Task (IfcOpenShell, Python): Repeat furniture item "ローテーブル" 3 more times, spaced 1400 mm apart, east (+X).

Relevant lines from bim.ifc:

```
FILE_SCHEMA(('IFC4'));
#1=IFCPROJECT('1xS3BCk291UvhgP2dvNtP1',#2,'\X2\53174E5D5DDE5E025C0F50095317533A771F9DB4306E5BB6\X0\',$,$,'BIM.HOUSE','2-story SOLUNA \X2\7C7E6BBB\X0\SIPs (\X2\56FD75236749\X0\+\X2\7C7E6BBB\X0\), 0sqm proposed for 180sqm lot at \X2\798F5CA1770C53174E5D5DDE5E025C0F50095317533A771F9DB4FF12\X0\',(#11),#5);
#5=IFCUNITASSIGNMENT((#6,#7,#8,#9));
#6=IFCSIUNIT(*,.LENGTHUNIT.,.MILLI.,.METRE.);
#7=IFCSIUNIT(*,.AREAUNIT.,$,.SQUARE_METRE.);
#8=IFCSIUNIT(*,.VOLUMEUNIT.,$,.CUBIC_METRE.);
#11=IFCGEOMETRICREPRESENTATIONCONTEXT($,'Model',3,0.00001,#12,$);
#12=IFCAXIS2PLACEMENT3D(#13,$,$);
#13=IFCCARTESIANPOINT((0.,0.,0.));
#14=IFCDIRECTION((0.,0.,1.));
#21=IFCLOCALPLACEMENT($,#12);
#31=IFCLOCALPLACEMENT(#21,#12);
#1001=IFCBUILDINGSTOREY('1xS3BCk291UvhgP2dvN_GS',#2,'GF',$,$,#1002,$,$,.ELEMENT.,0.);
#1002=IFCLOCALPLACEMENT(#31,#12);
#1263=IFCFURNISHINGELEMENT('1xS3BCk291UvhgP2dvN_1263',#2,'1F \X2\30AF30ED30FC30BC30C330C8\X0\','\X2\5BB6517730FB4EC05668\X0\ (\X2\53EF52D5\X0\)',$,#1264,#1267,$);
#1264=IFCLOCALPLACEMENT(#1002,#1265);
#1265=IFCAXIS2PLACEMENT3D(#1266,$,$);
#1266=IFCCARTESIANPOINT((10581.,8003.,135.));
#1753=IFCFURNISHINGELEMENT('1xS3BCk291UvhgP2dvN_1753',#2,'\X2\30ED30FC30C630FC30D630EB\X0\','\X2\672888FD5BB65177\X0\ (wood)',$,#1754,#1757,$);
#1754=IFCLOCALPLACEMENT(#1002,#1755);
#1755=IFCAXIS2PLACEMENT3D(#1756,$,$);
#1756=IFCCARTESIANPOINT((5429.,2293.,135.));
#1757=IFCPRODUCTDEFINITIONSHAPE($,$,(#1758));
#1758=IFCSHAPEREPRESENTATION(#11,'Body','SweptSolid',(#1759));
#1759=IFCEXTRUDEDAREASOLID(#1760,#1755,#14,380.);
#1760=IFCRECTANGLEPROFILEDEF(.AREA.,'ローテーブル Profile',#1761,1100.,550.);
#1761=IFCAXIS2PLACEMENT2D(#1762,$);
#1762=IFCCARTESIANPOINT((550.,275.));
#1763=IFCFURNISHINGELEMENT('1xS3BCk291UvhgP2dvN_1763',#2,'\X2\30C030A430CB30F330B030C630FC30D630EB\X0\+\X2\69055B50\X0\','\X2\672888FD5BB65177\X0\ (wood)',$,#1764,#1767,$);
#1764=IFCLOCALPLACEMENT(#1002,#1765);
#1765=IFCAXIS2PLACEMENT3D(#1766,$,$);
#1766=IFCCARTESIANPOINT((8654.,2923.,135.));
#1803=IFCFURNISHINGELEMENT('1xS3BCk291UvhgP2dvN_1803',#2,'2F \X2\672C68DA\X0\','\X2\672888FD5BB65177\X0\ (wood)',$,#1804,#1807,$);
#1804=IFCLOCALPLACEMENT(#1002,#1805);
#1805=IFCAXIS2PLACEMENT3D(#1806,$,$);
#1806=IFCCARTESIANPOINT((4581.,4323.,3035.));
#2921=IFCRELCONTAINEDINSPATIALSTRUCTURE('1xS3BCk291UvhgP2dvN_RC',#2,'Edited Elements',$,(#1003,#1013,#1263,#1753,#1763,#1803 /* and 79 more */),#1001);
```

```python
import numpy as np
import ifcopenshell
import ifcopenshell.api.geometry
import ifcopenshell.api.root
import ifcopenshell.util.element
import ifcopenshell.util.placement

model = ifcopenshell.open("bim.ifc")


def reuse_history(source, copy):
    """copy_class also copies each property set's owner history, people and application; keep the originals."""
    for rel in copy.IsDefinedBy:
        if rel.is_a("IfcRelDefinesByProperties") and (history := rel.RelatingPropertyDefinition.OwnerHistory):
            rel.RelatingPropertyDefinition.OwnerHistory = source.OwnerHistory
            ifcopenshell.util.element.remove_deep2(model, history)


source = model.by_guid("1xS3BCk291UvhgP2dvN_1753")
base = ifcopenshell.util.placement.get_local_placement(source.ObjectPlacement)
step = np.array([1.0, 0.0, 0.0]) * 1400.0

for i in range(1, 4):
    copy = ifcopenshell.api.root.copy_class(model, product=source)
    copy.Representation = ifcopenshell.util.element.copy_deep(
        model, source.Representation, exclude=["IfcGeometricRepresentationContext", "IfcRepresentationMap"]
    )
    reuse_history(source, copy)
    matrix = base.copy()
    matrix[:3, 3] += i * step
    print("added at", matrix[:3, 3].round(3) + 0.0)
    ifcopenshell.api.geometry.edit_object_placement(model, product=copy, matrix=matrix, is_si=False)

model.write("bim_updated.ifc")
```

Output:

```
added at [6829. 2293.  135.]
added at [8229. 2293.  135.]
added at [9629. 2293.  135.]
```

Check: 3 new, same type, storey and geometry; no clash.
